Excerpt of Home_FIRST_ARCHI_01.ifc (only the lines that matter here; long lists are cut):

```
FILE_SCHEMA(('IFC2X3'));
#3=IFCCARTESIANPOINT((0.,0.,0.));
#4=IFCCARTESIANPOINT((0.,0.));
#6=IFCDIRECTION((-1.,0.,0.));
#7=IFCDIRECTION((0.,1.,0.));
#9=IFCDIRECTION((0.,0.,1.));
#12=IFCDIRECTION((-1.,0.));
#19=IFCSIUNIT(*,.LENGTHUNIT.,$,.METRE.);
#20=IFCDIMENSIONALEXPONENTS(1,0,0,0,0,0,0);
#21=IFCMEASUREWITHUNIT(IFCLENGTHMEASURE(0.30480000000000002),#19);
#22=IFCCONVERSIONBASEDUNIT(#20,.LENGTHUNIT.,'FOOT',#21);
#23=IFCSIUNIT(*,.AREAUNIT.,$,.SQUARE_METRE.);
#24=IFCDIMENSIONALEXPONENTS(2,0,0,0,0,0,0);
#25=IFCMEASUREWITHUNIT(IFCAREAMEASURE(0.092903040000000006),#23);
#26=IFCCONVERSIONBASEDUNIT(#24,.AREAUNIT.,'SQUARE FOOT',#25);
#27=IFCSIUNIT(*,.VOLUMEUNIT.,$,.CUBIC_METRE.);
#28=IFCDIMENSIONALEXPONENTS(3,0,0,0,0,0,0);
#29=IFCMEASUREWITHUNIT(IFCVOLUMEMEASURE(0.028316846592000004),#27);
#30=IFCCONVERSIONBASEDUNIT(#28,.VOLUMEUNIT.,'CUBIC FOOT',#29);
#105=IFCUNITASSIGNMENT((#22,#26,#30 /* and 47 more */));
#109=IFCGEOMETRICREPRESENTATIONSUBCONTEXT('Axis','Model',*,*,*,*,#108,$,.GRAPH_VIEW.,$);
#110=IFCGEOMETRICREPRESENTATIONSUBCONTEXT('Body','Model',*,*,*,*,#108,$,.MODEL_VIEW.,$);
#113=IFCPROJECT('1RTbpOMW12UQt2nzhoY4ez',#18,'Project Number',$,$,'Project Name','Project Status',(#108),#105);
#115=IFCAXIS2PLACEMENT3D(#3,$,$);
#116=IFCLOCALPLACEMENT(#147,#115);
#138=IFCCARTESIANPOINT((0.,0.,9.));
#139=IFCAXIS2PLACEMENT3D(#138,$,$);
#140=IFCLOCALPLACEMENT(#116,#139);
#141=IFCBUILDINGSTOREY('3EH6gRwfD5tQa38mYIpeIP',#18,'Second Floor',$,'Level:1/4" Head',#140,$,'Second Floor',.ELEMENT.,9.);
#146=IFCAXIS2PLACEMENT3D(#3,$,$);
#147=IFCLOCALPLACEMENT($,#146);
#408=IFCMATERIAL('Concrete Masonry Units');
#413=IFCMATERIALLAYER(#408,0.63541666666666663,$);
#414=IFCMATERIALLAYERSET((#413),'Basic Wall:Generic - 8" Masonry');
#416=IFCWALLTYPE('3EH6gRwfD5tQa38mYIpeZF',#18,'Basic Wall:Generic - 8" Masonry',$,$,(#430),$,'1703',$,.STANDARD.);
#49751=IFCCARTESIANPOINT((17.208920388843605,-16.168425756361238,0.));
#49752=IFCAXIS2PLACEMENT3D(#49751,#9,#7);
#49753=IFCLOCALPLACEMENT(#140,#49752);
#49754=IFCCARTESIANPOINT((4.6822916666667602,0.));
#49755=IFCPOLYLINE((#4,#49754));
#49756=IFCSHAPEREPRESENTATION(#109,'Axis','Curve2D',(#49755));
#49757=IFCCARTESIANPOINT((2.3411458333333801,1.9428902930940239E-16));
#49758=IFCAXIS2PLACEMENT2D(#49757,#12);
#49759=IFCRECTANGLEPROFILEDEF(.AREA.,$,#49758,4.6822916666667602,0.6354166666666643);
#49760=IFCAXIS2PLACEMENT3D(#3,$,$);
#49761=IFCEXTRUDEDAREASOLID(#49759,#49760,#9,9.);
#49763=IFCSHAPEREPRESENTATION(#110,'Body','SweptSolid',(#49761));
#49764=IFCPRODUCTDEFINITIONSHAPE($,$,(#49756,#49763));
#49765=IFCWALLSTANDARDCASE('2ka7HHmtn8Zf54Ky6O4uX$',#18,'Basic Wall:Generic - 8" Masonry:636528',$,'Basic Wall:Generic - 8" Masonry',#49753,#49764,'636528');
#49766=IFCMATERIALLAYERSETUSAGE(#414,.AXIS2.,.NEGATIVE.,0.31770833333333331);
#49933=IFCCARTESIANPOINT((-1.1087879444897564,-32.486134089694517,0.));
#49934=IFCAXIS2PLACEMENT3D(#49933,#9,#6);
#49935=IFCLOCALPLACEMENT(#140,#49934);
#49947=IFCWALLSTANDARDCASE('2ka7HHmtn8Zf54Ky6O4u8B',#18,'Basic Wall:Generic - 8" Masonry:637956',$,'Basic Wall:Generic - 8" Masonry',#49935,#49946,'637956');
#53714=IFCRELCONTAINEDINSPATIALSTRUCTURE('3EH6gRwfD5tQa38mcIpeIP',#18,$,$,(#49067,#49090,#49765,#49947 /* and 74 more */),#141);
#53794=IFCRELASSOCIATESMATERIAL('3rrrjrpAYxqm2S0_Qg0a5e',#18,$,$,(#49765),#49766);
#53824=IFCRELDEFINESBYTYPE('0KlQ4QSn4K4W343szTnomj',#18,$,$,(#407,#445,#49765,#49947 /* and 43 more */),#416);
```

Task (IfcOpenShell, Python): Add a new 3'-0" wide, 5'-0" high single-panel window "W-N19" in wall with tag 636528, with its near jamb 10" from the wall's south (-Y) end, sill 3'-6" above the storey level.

```python
import numpy as np
import ifcopenshell
import ifcopenshell.api.feature
import ifcopenshell.api.geometry
import ifcopenshell.api.root
import ifcopenshell.api.spatial
import ifcopenshell.api.type
import ifcopenshell.geom
import ifcopenshell.util.element
import ifcopenshell.util.placement
import ifcopenshell.util.representation
import ifcopenshell.util.shape
import ifcopenshell.util.unit

model = ifcopenshell.open("Home_FIRST_ARCHI_01.ifc")
unit_scale = ifcopenshell.util.unit.calculate_unit_scale(model)
settings = ifcopenshell.geom.settings()


def volume(element):
    """Net volume in cubic metres, openings subtracted."""
    shape = ifcopenshell.geom.create_shape(settings, element)
    return ifcopenshell.util.shape.get_volume(shape.geometry)


wall = model.by_id(49765)
storey = ifcopenshell.util.element.get_container(wall, ifc_class="IfcBuildingStorey")
context = ifcopenshell.util.representation.get_context(model, "Model", "Body", "MODEL_VIEW")
before = volume(wall)

width, height, from_end, sill = 0.9144, 1.524, 0.254, 1.0668  # metres

# The wall runs along its own X axis, and the end named is its -X end.
wall_shape = ifcopenshell.geom.create_shape(settings, wall)
x, y, z = ifcopenshell.util.shape.get_vertices(wall_shape.geometry).T
start = x.min() + from_end
face, thickness = float(y.min()), float(y.max() - y.min())
wall_matrix = ifcopenshell.util.placement.get_local_placement(wall.ObjectPlacement)
level = ifcopenshell.util.placement.get_local_placement(storey.ObjectPlacement)[2, 3]


def in_wall(x, y):
    """Placement at x, y metres in the wall's axes, at sill height."""
    matrix = wall_matrix.copy()
    matrix[:, 3] = wall_matrix @ np.array([x / unit_scale, y / unit_scale, 0.0, 1.0])
    matrix[2, 3] = level + sill / unit_scale
    return matrix


# Opening: a box that overshoots both wall faces by 50 mm.
opening = ifcopenshell.api.root.create_entity(model, ifc_class="IfcOpeningElement")
box = ifcopenshell.api.geometry.add_wall_representation(
    model, context=context, length=width, height=height, thickness=thickness + 0.1
)
ifcopenshell.api.geometry.assign_representation(model, product=opening, representation=box)
ifcopenshell.api.geometry.edit_object_placement(model, product=opening, matrix=in_wall(start, face - 0.05), is_si=False)
ifcopenshell.api.feature.add_feature(model, feature=opening, element=wall)

window = ifcopenshell.api.root.create_entity(model, ifc_class="IfcWindow", name="W-N19")
window.OverallWidth, window.OverallHeight = width / unit_scale, height / unit_scale
body = ifcopenshell.api.geometry.add_window_representation(
    model,
    context=context,
    overall_width=window.OverallWidth,
    overall_height=window.OverallHeight,
    partition_type="SINGLE_PANEL",
)
ifcopenshell.api.geometry.assign_representation(model, product=window, representation=body)
ifcopenshell.api.spatial.assign_container(model, products=[window], relating_structure=storey)
fills = ifcopenshell.api.feature.add_filling(model, opening=opening, element=window)
fills.OwnerHistory = window.OwnerHistory  # required in IFC2X3

# IFC2X3 keeps the operation on the window style.
style = ifcopenshell.api.root.create_entity(model, ifc_class="IfcWindowStyle", name="W-N19")
style.OperationType, style.ConstructionType = "SINGLE_PANEL", "NOTDEFINED"
style.ParameterTakesPrecedence = style.Sizeable = False
ifcopenshell.api.type.assign_type(model, related_objects=[window], relating_type=style)

# Centre the window in the wall's thickness.
ifcopenshell.api.geometry.edit_object_placement(model, product=window, matrix=in_wall(start, face), is_si=False)
window_shape = ifcopenshell.geom.create_shape(settings, window)
depth = ifcopenshell.util.shape.get_vertices(window_shape.geometry)[:, 1]
offset = face + thickness / 2 - (depth.min() + depth.max()) / 2
ifcopenshell.api.geometry.edit_object_placement(model, product=window, matrix=in_wall(start, offset), is_si=False)

after = volume(wall)

print(f"wall volume {before:.3f} -> {after:.3f} m3")

model.write("Home_FIRST_ARCHI_01_edited.ifc")
```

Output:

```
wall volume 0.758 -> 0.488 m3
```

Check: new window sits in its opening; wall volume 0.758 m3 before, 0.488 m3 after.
